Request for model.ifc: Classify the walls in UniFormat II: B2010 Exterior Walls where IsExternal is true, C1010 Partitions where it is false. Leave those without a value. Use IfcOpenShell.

First a look at what the model holds.

```python
import ifcopenshell
import ifcopenshell.util.element

model = ifcopenshell.open("model.ifc")
print(model.schema)
print("classifications:", [c.Name for c in model.by_type("IfcClassification")])
values = [ifcopenshell.util.element.get_pset(e, "Pset_WallCommon", "IsExternal") for e in model.by_type("IfcWall")]
for value in (True, False, None):
    print("IsExternal", value, values.count(value))
```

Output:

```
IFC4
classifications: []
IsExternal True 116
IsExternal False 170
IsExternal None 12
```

```python
import ifcopenshell
import ifcopenshell.api.classification
import ifcopenshell.util.element

model = ifcopenshell.open("model.ifc")

system = ifcopenshell.api.classification.add_classification(model, classification="UniFormat II")

walls = model.by_type("IfcWall")
external = {e: ifcopenshell.util.element.get_pset(e, "Pset_WallCommon", "IsExternal") for e in walls}
for flag, code, name in ((True, "B2010", "Exterior Walls"), (False, "C1010", "Partitions")):
    products = [e for e in walls if external[e] is flag]
    ifcopenshell.api.classification.add_reference(
        model, products=products, classification=system, identification=code, name=name
    )
    print(code, len(products))

model.write("model_v2.ifc")
```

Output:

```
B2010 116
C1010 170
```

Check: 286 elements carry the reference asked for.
